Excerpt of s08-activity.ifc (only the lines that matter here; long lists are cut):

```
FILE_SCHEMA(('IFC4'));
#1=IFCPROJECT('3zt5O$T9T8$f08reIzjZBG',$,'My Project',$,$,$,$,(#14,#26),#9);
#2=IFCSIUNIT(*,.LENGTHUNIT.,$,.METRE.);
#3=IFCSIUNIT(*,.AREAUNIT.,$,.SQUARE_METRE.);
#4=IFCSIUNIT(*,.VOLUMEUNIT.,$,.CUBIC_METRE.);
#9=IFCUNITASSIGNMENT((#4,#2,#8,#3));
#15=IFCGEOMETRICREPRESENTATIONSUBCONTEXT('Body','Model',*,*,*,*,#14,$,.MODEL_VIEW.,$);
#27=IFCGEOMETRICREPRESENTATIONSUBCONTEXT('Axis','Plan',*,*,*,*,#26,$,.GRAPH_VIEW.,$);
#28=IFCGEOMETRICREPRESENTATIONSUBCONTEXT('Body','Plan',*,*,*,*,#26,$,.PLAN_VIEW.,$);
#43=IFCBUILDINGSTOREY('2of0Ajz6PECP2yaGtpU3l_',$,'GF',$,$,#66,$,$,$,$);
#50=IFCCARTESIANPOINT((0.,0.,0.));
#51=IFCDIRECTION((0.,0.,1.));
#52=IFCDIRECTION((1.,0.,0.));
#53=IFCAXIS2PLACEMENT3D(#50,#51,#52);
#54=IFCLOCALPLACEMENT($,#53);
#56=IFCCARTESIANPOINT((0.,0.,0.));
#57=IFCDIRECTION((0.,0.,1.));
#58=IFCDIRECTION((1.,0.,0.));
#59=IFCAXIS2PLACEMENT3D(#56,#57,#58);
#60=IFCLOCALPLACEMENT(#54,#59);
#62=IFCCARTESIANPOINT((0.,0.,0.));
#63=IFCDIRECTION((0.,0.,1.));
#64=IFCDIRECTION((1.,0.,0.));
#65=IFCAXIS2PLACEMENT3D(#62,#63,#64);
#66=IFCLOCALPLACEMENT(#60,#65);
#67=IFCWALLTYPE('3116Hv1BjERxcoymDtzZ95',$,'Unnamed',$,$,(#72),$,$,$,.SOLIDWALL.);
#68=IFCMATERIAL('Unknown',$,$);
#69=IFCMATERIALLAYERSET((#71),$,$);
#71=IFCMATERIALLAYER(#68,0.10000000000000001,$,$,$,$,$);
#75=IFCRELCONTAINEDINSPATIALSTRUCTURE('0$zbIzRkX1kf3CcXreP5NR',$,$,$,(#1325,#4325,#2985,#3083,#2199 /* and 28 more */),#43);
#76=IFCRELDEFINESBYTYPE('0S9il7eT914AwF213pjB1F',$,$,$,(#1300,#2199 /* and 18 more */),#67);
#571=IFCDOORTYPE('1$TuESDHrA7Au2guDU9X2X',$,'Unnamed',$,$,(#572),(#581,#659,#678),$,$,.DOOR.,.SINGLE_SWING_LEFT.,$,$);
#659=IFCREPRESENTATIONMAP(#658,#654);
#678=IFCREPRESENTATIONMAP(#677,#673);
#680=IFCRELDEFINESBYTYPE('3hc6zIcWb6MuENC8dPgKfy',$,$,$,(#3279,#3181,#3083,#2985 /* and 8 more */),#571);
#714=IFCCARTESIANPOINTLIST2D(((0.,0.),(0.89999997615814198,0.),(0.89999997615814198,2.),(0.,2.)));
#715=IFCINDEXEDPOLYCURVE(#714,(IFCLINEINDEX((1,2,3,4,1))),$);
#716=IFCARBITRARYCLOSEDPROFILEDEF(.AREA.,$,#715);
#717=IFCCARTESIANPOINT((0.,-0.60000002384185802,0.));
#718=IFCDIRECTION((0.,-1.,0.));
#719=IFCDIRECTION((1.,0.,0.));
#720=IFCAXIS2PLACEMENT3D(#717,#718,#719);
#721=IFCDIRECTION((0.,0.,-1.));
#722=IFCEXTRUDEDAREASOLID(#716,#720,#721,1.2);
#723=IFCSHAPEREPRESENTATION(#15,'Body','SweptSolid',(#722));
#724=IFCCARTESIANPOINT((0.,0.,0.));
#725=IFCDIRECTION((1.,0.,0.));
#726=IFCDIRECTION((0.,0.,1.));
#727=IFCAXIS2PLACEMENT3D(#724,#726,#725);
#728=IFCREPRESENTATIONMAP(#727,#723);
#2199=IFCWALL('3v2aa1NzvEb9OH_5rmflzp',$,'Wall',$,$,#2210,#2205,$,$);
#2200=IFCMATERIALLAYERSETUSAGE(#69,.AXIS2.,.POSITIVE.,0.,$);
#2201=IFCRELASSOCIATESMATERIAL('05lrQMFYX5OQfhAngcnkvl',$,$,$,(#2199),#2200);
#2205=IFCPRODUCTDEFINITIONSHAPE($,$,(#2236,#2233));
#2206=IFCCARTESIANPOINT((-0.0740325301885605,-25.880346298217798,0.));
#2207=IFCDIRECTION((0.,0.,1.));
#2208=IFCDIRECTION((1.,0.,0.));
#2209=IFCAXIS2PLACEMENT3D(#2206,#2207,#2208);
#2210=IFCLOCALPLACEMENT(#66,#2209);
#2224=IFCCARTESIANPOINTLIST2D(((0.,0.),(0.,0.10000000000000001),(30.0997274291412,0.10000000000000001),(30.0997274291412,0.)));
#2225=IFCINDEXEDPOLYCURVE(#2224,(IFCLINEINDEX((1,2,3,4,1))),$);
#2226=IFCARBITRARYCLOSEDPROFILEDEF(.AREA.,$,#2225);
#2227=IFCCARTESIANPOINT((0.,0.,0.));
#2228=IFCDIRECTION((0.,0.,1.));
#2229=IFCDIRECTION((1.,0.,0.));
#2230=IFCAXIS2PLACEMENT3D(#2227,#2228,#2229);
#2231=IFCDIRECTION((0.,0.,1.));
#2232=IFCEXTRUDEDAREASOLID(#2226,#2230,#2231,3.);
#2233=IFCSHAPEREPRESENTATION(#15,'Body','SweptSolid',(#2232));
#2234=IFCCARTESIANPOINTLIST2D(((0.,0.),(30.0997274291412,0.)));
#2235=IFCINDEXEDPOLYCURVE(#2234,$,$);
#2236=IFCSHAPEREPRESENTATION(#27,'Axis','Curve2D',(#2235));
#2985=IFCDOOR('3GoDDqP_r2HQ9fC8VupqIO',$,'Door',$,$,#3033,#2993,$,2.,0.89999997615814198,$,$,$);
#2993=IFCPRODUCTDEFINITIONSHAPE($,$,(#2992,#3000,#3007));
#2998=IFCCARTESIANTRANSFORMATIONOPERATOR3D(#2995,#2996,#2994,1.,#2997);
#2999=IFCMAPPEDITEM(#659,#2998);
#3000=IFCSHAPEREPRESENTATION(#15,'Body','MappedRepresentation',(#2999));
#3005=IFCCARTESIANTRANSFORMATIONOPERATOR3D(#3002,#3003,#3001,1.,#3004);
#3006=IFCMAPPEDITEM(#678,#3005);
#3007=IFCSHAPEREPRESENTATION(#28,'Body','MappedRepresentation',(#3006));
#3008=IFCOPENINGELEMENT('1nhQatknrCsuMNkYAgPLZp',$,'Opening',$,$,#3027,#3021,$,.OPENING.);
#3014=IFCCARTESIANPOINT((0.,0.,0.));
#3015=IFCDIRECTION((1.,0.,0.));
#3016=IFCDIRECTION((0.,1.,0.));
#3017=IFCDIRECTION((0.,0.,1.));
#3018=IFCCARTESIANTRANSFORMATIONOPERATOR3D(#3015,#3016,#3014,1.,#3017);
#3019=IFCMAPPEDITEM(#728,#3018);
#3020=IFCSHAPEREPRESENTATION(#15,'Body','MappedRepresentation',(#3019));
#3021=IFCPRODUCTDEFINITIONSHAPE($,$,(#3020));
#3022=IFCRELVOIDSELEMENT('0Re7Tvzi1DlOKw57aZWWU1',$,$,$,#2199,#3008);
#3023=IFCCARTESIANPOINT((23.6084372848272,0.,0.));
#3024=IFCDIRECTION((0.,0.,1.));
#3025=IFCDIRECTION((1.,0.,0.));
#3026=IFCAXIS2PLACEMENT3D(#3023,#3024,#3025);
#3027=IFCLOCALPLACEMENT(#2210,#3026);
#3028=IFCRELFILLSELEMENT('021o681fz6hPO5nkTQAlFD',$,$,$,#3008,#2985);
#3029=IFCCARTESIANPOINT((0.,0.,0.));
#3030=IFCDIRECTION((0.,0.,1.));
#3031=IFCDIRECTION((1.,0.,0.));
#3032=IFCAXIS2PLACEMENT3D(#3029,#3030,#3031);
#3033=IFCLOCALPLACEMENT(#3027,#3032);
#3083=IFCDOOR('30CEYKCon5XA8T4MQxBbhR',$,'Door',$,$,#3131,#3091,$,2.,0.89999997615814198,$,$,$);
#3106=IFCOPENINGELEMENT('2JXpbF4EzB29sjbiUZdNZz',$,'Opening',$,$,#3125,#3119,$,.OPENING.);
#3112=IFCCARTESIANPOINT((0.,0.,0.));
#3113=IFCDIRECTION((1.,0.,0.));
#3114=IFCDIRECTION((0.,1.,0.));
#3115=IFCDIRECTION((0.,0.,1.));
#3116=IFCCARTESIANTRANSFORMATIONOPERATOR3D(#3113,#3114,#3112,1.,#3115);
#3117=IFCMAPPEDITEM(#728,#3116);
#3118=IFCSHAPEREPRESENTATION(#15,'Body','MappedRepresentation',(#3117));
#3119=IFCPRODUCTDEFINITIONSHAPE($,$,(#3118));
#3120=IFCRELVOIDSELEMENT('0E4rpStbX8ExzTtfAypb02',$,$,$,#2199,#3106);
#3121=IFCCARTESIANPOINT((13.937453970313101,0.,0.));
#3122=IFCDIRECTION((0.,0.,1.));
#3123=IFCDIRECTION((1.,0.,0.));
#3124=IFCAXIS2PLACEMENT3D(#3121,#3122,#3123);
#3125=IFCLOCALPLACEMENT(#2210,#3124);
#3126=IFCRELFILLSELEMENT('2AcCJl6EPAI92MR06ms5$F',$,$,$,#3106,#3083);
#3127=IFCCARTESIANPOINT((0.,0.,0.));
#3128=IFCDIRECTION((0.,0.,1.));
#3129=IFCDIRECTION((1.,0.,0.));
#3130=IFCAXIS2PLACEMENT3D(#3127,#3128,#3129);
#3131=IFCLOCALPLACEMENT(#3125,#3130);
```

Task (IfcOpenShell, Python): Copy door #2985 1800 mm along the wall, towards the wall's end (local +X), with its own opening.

```python
import ifcopenshell
import ifcopenshell.api.feature
import ifcopenshell.api.geometry
import ifcopenshell.api.root
import ifcopenshell.geom
import ifcopenshell.util.element
import ifcopenshell.util.placement
import ifcopenshell.util.shape
import ifcopenshell.util.unit

model = ifcopenshell.open("s08-activity.ifc")
unit_scale = ifcopenshell.util.unit.calculate_unit_scale(model)
settings = ifcopenshell.geom.settings()


def volume(element):
    """Net volume in cubic metres, openings subtracted."""
    shape = ifcopenshell.geom.create_shape(settings, element)
    return ifcopenshell.util.shape.get_volume(shape.geometry)


door = model.by_guid("3GoDDqP_r2HQ9fC8VupqIO")
opening = door.FillsVoids[0].RelatingOpeningElement
wall = opening.VoidsElements[0].RelatingBuildingElement
before = volume(wall)
shift = ifcopenshell.util.placement.get_local_placement(wall.ObjectPlacement)[:3, 0] * 1.8 / unit_scale

# copy_class copies the void relationship, type, container and properties, but no geometry.
new_opening = ifcopenshell.api.root.copy_class(model, product=opening)
new_opening.Representation = ifcopenshell.util.element.copy_deep(
    model, opening.Representation, exclude=["IfcGeometricRepresentationContext", "IfcRepresentationMap"]
)
new_door = ifcopenshell.api.root.copy_class(model, product=door)
new_door.Representation = ifcopenshell.util.element.copy_deep(
    model, door.Representation, exclude=["IfcGeometricRepresentationContext", "IfcRepresentationMap"]
)
ifcopenshell.api.feature.add_filling(model, opening=new_opening, element=new_door)

for old, new in ((opening, new_opening), (door, new_door)):
    matrix = ifcopenshell.util.placement.get_local_placement(old.ObjectPlacement)
    matrix[:3, 3] += shift
    ifcopenshell.api.geometry.edit_object_placement(model, product=new, matrix=matrix, is_si=False)

after = volume(wall)

print(f"wall volume {before:.3f} -> {after:.3f} m3")

model.write("s08-activity_edited.ifc")
```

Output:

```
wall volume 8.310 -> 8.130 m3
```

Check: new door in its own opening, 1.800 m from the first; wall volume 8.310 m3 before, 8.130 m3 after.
